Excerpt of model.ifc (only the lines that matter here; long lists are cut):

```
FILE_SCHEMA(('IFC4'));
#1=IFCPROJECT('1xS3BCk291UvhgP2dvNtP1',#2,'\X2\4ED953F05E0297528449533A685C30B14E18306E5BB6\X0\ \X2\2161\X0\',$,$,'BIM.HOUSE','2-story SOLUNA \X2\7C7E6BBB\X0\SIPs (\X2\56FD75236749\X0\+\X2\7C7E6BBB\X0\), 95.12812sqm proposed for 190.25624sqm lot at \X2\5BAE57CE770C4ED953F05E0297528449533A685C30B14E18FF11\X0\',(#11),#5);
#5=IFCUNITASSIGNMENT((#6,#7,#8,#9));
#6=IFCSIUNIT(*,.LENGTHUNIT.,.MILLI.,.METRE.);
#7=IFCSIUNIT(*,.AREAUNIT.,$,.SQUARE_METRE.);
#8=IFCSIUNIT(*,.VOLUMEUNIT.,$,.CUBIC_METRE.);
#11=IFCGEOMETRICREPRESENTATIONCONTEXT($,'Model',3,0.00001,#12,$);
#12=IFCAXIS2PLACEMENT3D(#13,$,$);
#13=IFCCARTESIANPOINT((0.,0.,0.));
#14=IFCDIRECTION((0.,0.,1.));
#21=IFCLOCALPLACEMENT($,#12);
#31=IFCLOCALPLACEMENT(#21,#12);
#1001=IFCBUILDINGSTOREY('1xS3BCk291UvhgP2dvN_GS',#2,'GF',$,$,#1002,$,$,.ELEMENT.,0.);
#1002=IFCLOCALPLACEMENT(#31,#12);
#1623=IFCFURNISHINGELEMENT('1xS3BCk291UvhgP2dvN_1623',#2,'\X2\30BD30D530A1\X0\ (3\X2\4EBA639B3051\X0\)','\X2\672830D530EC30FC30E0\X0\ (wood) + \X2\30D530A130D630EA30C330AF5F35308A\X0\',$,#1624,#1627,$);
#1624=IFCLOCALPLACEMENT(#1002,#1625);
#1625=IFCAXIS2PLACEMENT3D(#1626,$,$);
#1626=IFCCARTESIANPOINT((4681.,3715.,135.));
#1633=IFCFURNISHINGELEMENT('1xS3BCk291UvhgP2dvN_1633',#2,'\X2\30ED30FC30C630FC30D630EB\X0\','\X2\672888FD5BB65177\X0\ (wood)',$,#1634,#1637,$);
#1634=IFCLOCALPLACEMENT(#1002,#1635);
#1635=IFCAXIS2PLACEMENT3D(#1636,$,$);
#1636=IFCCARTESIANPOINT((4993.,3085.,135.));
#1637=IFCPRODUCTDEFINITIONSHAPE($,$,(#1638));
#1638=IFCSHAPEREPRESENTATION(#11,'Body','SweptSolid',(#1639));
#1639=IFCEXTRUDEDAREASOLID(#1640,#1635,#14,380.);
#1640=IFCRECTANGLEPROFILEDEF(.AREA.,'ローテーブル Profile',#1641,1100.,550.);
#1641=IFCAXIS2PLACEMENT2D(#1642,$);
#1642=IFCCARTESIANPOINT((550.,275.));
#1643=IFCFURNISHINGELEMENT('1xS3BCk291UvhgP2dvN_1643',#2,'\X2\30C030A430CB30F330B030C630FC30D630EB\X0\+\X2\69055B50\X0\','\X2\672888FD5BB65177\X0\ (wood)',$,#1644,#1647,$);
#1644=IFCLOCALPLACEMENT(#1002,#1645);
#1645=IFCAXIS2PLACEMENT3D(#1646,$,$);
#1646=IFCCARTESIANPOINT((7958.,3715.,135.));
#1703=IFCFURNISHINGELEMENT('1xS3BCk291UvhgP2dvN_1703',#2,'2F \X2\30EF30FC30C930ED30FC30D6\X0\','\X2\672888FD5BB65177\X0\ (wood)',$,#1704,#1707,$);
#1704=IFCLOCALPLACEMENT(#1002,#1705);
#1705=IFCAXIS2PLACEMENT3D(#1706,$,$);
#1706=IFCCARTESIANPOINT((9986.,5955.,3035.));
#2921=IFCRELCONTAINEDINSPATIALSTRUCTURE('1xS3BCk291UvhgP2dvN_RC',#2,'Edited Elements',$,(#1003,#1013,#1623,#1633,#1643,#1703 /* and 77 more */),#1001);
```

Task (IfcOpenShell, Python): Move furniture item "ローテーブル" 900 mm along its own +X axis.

```python
import ifcopenshell
import ifcopenshell.api.geometry
import ifcopenshell.util.placement

model = ifcopenshell.open("model.ifc")

item = model.by_guid("1xS3BCk291UvhgP2dvN_1633")
matrix = ifcopenshell.util.placement.get_local_placement(item.ObjectPlacement)
matrix[:3, 3] += matrix[:3, 0] * 900.0
ifcopenshell.api.geometry.edit_object_placement(model, product=item, matrix=matrix, is_si=False)

print(ifcopenshell.util.placement.get_local_placement(item.ObjectPlacement).round(3) + 0.0)

model.write("model-out.ifc")
```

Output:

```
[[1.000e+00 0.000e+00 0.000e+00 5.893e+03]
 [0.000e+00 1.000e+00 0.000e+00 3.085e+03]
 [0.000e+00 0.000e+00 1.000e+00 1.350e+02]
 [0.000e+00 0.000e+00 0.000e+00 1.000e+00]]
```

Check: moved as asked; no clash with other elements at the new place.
